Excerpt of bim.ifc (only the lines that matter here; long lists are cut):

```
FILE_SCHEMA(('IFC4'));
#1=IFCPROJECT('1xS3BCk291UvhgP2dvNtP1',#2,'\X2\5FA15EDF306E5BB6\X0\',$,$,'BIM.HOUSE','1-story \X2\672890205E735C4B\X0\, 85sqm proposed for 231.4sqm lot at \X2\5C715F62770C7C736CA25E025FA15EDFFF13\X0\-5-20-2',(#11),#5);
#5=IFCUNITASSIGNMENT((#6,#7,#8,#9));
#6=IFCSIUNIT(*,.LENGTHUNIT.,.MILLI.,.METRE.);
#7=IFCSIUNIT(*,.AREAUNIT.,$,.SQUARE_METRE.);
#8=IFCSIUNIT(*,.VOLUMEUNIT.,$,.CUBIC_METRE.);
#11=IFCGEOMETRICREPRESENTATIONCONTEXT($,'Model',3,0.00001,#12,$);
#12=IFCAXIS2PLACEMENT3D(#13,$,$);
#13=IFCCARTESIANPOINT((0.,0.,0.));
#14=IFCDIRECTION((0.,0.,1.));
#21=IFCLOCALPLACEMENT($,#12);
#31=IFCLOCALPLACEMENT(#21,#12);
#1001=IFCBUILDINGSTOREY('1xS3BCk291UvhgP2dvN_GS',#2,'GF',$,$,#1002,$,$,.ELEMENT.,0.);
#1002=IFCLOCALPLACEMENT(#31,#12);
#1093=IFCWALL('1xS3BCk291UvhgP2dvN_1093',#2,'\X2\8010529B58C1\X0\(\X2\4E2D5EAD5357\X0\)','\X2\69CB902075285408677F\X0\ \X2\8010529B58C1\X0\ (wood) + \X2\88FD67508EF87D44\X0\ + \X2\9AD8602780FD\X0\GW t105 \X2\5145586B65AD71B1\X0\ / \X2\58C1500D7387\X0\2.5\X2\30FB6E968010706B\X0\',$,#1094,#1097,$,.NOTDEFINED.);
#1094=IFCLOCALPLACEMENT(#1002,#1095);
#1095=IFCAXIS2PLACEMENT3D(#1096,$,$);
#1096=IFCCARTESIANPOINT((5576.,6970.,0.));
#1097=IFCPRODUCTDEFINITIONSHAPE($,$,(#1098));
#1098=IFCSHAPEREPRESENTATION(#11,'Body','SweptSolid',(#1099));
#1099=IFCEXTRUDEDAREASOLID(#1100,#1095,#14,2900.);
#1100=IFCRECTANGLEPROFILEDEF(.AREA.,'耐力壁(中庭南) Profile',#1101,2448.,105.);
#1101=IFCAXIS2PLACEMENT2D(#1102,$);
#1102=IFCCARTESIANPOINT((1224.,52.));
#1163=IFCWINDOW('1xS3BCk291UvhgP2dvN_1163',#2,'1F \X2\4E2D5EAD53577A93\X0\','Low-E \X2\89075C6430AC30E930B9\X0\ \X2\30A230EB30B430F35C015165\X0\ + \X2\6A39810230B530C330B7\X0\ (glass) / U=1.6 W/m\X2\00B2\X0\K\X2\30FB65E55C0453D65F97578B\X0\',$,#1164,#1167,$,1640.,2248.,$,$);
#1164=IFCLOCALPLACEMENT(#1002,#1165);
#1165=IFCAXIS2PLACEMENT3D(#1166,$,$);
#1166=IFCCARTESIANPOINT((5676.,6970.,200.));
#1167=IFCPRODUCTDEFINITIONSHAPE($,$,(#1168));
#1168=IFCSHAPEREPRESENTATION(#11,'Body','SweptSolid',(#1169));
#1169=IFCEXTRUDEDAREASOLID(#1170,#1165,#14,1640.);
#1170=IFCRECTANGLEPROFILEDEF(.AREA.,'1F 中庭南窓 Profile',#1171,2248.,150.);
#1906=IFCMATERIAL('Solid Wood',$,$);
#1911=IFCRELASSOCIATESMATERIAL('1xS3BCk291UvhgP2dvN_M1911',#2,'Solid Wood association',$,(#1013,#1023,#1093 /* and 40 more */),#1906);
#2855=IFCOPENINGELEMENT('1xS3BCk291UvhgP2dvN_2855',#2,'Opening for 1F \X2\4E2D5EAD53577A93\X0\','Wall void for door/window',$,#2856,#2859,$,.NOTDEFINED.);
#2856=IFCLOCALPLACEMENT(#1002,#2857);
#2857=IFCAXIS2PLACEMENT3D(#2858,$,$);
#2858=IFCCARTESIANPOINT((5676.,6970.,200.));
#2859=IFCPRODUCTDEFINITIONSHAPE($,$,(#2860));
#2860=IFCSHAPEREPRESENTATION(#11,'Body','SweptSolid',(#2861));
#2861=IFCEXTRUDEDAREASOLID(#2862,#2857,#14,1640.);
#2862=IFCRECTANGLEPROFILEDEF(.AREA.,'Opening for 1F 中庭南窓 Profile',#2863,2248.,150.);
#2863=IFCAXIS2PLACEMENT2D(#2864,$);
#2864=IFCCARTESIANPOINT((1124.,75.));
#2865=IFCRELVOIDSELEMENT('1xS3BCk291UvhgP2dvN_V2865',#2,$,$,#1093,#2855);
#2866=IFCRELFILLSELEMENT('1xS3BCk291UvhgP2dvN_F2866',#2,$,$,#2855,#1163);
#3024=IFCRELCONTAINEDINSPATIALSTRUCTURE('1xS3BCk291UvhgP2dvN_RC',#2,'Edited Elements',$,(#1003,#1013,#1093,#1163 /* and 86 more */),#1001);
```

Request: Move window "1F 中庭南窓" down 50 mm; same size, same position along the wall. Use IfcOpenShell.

```python
import numpy as np
import ifcopenshell
import ifcopenshell.api.geometry
import ifcopenshell.util.placement
import ifcopenshell.util.unit

model = ifcopenshell.open("bim.ifc")
unit_scale = ifcopenshell.util.unit.calculate_unit_scale(model)

window = model.by_id(1163)
opening = window.FillsVoids[0].RelatingOpeningElement
dz = -50.0

shift = np.array([0.0, 0.0, dz])
# The window is not placed relative to its opening, so move both.
for product in (opening, window):
    matrix = ifcopenshell.util.placement.get_local_placement(product.ObjectPlacement)
    matrix[:3, 3] += shift
    ifcopenshell.api.geometry.edit_object_placement(model, product=product, matrix=matrix, is_si=False)

print(f"moved by {dz * unit_scale:+.3f} m")

model.write("bim_updated.ifc")
```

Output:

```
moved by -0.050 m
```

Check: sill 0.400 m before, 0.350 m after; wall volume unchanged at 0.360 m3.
